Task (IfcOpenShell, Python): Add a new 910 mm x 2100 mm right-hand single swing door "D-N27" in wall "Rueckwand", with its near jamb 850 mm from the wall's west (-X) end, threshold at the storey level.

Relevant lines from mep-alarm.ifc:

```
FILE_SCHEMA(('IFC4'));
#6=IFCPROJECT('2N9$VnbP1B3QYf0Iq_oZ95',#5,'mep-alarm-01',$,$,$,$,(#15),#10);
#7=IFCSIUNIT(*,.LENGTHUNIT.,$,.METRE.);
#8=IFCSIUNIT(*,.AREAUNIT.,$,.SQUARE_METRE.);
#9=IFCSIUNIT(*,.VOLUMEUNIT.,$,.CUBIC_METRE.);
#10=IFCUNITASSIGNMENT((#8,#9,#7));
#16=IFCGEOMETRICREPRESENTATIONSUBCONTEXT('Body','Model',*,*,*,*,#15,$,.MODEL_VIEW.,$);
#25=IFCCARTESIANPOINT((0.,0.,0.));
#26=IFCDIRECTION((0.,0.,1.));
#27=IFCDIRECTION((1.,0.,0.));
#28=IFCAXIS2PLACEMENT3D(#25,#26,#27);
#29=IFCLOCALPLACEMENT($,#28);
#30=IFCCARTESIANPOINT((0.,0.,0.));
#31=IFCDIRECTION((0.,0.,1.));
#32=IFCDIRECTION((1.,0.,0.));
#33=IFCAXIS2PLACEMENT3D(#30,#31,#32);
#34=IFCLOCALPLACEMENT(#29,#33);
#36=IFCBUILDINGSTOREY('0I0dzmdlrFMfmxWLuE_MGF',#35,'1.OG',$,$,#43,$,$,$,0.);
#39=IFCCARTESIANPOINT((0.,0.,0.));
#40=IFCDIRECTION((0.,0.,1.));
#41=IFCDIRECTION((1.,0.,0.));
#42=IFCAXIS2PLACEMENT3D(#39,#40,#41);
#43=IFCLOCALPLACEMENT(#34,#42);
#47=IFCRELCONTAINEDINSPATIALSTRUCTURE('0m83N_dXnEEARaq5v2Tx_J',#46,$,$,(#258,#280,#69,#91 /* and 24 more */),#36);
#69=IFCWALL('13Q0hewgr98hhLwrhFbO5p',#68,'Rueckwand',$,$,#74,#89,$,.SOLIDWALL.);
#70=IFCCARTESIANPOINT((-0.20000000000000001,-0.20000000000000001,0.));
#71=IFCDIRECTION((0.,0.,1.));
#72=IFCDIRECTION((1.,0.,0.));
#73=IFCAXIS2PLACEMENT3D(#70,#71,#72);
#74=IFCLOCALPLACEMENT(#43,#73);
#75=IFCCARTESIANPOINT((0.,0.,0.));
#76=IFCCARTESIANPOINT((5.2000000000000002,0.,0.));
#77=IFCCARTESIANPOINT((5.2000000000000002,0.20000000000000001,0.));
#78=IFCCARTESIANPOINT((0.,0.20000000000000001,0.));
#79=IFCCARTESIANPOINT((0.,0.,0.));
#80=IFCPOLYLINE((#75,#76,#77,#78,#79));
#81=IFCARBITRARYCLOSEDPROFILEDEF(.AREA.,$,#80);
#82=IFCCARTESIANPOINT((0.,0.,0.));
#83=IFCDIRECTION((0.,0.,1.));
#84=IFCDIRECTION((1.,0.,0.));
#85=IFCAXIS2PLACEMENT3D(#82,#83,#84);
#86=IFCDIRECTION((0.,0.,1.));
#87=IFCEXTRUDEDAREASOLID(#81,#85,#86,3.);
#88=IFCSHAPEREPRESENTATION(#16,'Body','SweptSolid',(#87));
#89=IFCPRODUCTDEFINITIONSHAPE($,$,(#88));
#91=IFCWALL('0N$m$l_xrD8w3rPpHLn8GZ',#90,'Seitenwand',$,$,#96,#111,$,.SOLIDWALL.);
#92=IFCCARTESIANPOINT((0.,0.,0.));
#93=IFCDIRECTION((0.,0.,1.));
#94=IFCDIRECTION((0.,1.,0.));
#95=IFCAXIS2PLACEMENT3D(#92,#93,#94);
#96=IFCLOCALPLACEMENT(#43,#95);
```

```python
import numpy as np
import ifcopenshell
import ifcopenshell.api.feature
import ifcopenshell.api.geometry
import ifcopenshell.api.root
import ifcopenshell.api.spatial
import ifcopenshell.geom
import ifcopenshell.util.element
import ifcopenshell.util.placement
import ifcopenshell.util.representation
import ifcopenshell.util.shape
import ifcopenshell.util.unit

model = ifcopenshell.open("mep-alarm.ifc")
unit_scale = ifcopenshell.util.unit.calculate_unit_scale(model)
settings = ifcopenshell.geom.settings()


def volume(element):
    """Net volume in cubic metres, openings subtracted."""
    shape = ifcopenshell.geom.create_shape(settings, element)
    return ifcopenshell.util.shape.get_volume(shape.geometry)


wall = model.by_id(69)
storey = ifcopenshell.util.element.get_container(wall, ifc_class="IfcBuildingStorey")
context = ifcopenshell.util.representation.get_context(model, "Model", "Body", "MODEL_VIEW")
before = volume(wall)

width, height, from_end, sill = 0.91, 2.1, 0.85, 0.0  # metres

# The wall runs along its own X axis, and the end named is its -X end.
wall_shape = ifcopenshell.geom.create_shape(settings, wall)
x, y, z = ifcopenshell.util.shape.get_vertices(wall_shape.geometry).T
start = x.min() + from_end
face, thickness = float(y.min()), float(y.max() - y.min())
wall_matrix = ifcopenshell.util.placement.get_local_placement(wall.ObjectPlacement)
level = ifcopenshell.util.placement.get_local_placement(storey.ObjectPlacement)[2, 3]


def in_wall(x, y):
    """Placement at x, y metres in the wall's axes, at sill height."""
    matrix = wall_matrix.copy()
    matrix[:, 3] = wall_matrix @ np.array([x / unit_scale, y / unit_scale, 0.0, 1.0])
    matrix[2, 3] = level + sill / unit_scale
    return matrix


# Opening: a box that overshoots both wall faces by 50 mm.
opening = ifcopenshell.api.root.create_entity(model, ifc_class="IfcOpeningElement", predefined_type="OPENING")
box = ifcopenshell.api.geometry.add_wall_representation(
    model, context=context, length=width, height=height, thickness=thickness + 0.1
)
ifcopenshell.api.geometry.assign_representation(model, product=opening, representation=box)
ifcopenshell.api.geometry.edit_object_placement(model, product=opening, matrix=in_wall(start, face - 0.05), is_si=False)
ifcopenshell.api.feature.add_feature(model, feature=opening, element=wall)

door = ifcopenshell.api.root.create_entity(model, ifc_class="IfcDoor", name="D-N27", predefined_type="DOOR")
door.OverallWidth, door.OverallHeight = width / unit_scale, height / unit_scale
door.OperationType = "SINGLE_SWING_RIGHT"
body = ifcopenshell.api.geometry.add_door_representation(
    model,
    context=context,
    overall_width=door.OverallWidth,
    overall_height=door.OverallHeight,
    operation_type="SINGLE_SWING_RIGHT",
    lining_properties={"LiningDepth": thickness / unit_scale, "ThresholdDepth": thickness / unit_scale},
)
ifcopenshell.api.geometry.assign_representation(model, product=door, representation=body)
ifcopenshell.api.spatial.assign_container(model, products=[door], relating_structure=storey)
ifcopenshell.api.feature.add_filling(model, opening=opening, element=door)

# The lining spans the wall, so the door starts at the wall face.
ifcopenshell.api.geometry.edit_object_placement(model, product=door, matrix=in_wall(start, face), is_si=False)

after = volume(wall)

print(f"wall volume {before:.3f} -> {after:.3f} m3")

model.write("mep-alarm-out.ifc")
```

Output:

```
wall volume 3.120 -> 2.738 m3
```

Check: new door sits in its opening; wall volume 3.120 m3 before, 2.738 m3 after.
